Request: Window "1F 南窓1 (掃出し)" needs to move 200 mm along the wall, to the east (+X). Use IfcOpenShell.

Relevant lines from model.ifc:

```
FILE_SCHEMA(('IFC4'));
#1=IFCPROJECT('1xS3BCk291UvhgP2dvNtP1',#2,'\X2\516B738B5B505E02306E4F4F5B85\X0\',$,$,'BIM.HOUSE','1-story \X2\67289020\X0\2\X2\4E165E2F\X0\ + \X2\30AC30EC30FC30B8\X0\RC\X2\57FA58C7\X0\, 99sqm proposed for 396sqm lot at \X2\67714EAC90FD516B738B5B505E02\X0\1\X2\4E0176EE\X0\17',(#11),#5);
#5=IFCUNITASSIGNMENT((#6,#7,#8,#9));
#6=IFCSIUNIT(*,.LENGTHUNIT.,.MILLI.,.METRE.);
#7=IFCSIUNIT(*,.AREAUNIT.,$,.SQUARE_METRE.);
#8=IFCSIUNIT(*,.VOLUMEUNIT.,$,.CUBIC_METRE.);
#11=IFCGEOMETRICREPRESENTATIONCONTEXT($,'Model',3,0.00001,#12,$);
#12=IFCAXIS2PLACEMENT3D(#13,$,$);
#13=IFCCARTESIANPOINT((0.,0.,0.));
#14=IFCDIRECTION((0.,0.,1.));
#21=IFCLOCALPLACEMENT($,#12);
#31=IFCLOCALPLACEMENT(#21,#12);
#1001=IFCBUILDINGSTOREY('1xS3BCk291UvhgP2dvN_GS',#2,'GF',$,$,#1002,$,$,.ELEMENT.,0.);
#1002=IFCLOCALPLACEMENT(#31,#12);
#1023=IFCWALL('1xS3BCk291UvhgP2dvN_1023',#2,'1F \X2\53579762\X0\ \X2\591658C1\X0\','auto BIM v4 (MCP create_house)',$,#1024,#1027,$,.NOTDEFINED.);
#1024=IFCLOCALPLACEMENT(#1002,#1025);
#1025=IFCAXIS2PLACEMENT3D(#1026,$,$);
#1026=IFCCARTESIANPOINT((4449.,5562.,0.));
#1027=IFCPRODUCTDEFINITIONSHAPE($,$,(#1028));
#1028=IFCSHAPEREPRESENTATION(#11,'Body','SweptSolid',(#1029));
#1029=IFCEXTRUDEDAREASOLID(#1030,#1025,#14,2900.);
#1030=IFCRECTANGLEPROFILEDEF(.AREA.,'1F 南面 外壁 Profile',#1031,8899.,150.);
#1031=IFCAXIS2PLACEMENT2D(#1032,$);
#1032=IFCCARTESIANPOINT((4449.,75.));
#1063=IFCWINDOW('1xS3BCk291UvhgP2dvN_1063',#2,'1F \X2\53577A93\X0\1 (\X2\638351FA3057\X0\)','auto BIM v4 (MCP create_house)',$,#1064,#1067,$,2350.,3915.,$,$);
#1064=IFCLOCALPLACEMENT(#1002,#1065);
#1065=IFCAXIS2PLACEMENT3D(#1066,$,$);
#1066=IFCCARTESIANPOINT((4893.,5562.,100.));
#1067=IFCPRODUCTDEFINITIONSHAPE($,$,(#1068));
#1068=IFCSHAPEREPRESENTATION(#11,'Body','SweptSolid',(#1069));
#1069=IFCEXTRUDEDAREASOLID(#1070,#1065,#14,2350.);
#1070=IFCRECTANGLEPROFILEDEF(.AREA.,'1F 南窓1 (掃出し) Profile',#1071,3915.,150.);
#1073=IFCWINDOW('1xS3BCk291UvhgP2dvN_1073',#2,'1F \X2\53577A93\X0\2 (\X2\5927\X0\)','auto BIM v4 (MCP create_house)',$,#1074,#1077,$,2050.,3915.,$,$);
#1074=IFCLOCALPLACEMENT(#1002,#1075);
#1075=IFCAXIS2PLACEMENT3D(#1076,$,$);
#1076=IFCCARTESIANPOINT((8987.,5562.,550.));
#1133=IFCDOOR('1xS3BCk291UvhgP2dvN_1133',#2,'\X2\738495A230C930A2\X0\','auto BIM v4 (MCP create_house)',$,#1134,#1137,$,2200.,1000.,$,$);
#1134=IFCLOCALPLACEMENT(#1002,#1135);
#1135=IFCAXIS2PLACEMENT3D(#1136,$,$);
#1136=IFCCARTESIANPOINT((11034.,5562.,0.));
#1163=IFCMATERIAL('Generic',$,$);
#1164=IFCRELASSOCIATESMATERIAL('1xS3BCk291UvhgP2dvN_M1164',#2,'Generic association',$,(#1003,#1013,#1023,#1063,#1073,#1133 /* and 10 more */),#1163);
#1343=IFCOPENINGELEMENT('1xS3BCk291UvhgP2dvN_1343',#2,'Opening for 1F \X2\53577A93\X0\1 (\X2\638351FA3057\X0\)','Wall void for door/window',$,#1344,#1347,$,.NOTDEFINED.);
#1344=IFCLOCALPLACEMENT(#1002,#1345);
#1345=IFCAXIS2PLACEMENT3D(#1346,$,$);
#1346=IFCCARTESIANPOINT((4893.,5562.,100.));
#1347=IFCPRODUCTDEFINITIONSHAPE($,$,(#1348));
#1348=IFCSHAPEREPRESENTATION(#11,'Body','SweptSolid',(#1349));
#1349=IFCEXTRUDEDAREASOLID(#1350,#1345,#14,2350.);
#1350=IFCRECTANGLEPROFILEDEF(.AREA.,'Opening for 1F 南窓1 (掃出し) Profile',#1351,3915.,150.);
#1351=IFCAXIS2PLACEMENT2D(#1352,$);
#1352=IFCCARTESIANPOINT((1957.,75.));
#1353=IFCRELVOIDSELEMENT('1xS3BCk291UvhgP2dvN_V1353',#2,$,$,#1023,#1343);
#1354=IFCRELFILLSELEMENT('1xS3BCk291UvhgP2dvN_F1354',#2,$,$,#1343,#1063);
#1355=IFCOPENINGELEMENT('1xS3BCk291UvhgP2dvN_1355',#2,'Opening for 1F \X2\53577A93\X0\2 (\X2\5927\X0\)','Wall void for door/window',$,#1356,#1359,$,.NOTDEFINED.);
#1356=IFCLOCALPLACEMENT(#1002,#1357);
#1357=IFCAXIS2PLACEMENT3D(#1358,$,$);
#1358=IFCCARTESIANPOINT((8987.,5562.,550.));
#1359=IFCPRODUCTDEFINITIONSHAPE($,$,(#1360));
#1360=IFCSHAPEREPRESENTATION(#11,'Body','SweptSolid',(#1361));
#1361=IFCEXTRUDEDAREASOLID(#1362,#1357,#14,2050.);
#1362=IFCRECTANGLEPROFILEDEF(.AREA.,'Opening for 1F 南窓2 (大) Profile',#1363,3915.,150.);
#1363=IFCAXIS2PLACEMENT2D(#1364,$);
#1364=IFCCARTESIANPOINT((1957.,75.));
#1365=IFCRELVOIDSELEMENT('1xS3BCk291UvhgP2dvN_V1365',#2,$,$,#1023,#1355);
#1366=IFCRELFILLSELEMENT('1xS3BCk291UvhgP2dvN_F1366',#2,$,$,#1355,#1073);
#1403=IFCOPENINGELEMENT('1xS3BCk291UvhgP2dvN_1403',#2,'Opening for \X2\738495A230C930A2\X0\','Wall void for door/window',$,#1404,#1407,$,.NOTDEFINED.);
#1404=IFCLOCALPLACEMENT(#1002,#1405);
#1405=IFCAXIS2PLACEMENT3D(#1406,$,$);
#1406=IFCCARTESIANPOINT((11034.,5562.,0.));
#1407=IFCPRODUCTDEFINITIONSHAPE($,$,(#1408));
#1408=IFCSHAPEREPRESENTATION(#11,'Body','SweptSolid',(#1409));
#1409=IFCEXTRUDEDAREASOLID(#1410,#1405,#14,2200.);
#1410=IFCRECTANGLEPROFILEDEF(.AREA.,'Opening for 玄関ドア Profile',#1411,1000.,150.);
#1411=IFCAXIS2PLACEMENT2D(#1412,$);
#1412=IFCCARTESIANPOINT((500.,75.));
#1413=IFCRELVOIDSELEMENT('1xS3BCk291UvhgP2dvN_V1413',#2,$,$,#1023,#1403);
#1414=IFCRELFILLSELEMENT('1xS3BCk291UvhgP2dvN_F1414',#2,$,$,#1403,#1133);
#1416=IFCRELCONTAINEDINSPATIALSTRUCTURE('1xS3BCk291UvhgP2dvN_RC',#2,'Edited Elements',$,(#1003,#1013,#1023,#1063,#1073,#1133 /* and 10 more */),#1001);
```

```python
import ifcopenshell
import ifcopenshell.api.geometry
import ifcopenshell.util.placement

model = ifcopenshell.open("model.ifc")

window = model.by_id(1063)
opening = window.FillsVoids[0].RelatingOpeningElement
wall = opening.VoidsElements[0].RelatingBuildingElement

wall_matrix = ifcopenshell.util.placement.get_local_placement(wall.ObjectPlacement)
shift = wall_matrix[:3, 0] * 200.0
before = ifcopenshell.util.placement.get_local_placement(window.ObjectPlacement)[:3, 3].copy()

# The window is not placed relative to its opening, so move both.
for product in (opening, window):
    matrix = ifcopenshell.util.placement.get_local_placement(product.ObjectPlacement)
    matrix[:3, 3] += shift
    ifcopenshell.api.geometry.edit_object_placement(model, product=product, matrix=matrix, is_si=False)

after = ifcopenshell.util.placement.get_local_placement(window.ObjectPlacement)[:3, 3]
print("window moved by", (after - before).round(3) + 0.0)

model.write("model_rev.ifc")
```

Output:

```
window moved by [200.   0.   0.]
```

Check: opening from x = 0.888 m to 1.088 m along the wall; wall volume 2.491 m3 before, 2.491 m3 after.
